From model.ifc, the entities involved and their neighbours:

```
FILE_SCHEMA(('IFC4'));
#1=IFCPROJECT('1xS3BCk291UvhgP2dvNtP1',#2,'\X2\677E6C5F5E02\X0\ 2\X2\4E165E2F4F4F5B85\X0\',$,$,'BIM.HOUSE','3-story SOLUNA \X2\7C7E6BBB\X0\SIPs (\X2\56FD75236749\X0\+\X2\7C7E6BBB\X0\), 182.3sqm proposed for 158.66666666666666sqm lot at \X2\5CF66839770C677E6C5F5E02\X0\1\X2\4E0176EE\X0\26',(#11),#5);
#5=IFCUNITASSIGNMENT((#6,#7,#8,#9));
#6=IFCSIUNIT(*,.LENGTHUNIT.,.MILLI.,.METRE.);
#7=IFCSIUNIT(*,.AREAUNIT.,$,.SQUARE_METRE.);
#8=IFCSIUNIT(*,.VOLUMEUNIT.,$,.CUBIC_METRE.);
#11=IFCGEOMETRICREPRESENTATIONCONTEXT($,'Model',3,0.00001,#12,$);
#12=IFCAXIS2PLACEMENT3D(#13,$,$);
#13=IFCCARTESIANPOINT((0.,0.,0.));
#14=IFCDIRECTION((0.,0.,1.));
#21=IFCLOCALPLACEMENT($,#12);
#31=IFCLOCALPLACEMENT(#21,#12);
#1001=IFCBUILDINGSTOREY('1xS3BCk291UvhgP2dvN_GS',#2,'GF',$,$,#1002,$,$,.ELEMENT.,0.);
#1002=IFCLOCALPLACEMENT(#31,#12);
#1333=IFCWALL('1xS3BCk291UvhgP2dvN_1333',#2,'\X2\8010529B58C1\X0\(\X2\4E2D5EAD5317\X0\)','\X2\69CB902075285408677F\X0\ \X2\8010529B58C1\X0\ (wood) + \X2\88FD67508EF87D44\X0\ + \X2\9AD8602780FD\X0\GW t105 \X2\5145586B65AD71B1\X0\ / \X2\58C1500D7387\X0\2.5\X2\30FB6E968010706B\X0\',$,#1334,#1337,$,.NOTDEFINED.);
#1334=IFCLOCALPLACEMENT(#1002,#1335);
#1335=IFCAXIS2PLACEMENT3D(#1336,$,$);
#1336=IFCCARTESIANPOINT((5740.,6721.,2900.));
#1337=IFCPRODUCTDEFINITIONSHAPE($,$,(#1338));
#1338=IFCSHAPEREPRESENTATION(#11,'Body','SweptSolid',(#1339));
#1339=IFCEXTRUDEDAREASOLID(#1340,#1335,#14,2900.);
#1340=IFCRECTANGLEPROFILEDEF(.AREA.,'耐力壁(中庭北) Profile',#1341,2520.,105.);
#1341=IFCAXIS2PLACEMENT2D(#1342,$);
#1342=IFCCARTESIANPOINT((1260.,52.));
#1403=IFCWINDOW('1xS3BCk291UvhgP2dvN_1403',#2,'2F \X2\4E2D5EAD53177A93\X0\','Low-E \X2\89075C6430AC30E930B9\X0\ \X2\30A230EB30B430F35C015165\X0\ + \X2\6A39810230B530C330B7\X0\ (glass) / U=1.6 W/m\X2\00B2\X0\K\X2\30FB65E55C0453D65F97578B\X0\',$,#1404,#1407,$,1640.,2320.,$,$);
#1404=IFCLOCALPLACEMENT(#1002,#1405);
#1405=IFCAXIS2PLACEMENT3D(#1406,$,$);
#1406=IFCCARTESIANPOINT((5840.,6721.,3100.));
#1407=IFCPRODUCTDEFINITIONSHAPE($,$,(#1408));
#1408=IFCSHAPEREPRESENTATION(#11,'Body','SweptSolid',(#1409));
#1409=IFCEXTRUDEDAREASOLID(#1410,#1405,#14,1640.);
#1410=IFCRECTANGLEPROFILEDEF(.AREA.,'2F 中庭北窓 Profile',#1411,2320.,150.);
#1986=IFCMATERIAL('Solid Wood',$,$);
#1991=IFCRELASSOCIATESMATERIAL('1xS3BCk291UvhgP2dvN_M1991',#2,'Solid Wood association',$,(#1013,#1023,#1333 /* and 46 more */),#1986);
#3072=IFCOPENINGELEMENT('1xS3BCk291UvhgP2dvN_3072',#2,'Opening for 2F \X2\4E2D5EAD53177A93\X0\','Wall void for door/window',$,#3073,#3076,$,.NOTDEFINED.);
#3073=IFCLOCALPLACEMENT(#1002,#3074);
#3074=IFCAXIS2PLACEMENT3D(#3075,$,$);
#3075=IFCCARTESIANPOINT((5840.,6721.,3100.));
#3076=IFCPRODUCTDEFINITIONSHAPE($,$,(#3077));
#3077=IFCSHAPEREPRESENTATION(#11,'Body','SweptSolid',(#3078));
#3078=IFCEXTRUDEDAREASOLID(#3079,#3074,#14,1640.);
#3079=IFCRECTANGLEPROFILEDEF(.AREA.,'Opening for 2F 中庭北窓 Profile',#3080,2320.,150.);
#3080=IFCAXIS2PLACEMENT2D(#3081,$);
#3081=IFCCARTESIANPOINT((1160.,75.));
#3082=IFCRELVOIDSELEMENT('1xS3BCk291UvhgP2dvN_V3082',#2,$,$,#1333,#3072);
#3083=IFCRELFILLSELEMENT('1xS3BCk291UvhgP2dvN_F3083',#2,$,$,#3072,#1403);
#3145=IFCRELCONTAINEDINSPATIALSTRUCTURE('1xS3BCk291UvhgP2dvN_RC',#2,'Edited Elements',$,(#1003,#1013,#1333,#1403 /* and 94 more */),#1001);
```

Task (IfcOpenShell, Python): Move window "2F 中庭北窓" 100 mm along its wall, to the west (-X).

```python
import ifcopenshell
import ifcopenshell.api.geometry
import ifcopenshell.util.placement

model = ifcopenshell.open("model.ifc")

window = model.by_guid("1xS3BCk291UvhgP2dvN_1403")
opening = window.FillsVoids[0].RelatingOpeningElement
wall = opening.VoidsElements[0].RelatingBuildingElement

wall_matrix = ifcopenshell.util.placement.get_local_placement(wall.ObjectPlacement)
shift = wall_matrix[:3, 0] * -100.0
before = ifcopenshell.util.placement.get_local_placement(window.ObjectPlacement)[:3, 3].copy()

# The window is not placed relative to its opening, so move both.
for product in (opening, window):
    matrix = ifcopenshell.util.placement.get_local_placement(product.ObjectPlacement)
    matrix[:3, 3] += shift
    ifcopenshell.api.geometry.edit_object_placement(model, product=product, matrix=matrix, is_si=False)

after = ifcopenshell.util.placement.get_local_placement(window.ObjectPlacement)[:3, 3]
print("window moved by", (after - before).round(3) + 0.0)

model.write("model_rev.ifc")
```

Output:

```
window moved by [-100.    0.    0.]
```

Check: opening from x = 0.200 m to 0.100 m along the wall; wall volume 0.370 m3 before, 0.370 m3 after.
